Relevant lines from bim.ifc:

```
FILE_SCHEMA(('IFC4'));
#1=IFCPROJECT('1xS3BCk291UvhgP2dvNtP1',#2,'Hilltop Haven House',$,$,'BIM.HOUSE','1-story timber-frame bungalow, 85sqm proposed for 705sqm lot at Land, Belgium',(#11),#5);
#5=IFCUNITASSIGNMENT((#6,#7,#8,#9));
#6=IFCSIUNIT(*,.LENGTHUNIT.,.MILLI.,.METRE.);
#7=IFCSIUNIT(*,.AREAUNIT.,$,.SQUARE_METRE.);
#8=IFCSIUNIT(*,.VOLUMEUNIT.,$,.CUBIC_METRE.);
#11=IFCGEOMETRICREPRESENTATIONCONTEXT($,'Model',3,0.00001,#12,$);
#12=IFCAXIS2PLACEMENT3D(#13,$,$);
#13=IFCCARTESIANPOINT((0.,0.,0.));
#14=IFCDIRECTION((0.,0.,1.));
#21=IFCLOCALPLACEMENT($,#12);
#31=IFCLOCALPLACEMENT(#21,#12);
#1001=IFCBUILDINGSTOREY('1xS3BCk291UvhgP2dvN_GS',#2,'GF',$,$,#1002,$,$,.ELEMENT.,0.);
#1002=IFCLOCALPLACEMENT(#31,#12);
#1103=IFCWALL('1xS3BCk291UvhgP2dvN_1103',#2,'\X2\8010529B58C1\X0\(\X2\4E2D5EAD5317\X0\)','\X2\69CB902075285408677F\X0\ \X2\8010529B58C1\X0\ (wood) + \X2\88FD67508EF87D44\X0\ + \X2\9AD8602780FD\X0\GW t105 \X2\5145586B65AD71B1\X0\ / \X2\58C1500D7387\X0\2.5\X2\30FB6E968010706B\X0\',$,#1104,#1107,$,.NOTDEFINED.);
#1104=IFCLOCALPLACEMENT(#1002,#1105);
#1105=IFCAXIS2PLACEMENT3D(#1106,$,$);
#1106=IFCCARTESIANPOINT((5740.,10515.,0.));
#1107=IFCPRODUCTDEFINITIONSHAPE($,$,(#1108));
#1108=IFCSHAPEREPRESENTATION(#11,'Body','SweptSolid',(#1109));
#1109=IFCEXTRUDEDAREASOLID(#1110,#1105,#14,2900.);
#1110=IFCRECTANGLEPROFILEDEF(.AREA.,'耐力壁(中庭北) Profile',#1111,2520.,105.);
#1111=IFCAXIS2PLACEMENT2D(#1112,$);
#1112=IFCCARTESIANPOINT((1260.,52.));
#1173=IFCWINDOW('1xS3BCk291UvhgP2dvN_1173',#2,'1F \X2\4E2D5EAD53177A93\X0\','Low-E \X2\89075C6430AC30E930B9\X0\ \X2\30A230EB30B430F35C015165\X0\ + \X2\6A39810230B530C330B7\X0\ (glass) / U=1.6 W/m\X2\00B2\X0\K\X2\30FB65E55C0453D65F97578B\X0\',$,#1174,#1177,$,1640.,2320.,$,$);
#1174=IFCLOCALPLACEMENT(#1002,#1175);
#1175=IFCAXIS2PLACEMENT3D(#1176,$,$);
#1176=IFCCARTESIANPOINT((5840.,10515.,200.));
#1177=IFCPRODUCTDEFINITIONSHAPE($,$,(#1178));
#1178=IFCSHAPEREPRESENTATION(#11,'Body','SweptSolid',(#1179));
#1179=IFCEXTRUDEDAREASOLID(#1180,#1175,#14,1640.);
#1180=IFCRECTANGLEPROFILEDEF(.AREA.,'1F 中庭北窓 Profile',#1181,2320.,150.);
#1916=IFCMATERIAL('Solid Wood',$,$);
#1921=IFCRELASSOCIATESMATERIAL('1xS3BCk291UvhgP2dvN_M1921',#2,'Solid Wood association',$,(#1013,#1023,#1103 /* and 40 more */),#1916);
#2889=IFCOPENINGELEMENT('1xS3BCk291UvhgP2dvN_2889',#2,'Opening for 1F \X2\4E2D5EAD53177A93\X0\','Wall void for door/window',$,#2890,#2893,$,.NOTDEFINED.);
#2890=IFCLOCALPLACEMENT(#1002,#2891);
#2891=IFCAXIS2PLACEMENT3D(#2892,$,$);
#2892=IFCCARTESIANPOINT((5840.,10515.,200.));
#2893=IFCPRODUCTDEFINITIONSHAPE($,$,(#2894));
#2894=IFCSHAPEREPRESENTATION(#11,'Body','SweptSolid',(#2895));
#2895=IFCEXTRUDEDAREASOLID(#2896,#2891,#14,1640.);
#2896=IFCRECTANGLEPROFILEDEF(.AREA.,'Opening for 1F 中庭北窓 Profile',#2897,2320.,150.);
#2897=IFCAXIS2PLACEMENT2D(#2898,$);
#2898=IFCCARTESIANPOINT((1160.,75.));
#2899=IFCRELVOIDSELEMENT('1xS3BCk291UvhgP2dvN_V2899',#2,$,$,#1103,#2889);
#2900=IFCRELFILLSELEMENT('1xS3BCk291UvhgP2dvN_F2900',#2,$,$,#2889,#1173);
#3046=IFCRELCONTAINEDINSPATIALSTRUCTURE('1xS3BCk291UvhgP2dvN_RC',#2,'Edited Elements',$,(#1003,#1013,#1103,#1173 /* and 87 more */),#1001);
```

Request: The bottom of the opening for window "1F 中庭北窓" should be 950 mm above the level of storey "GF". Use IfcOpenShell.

```python
import numpy as np
import ifcopenshell
import ifcopenshell.api.geometry
import ifcopenshell.geom
import ifcopenshell.util.element
import ifcopenshell.util.placement
import ifcopenshell.util.shape
import ifcopenshell.util.unit

model = ifcopenshell.open("bim.ifc")
unit_scale = ifcopenshell.util.unit.calculate_unit_scale(model)

window = model.by_guid("1xS3BCk291UvhgP2dvN_1173")
opening = window.FillsVoids[0].RelatingOpeningElement
storey = ifcopenshell.util.element.get_container(window, ifc_class="IfcBuildingStorey")
level = ifcopenshell.util.placement.get_local_placement(storey.ObjectPlacement)[2, 3]

# The opening's origin need not be at the sill, so measure its lowest point.
shape = ifcopenshell.geom.create_shape(ifcopenshell.geom.settings(), opening)
bottom = ifcopenshell.util.shape.get_shape_bottom_elevation(shape, shape.geometry) / unit_scale
dz = level + 950.0 - bottom

shift = np.array([0.0, 0.0, dz])
# The window is not placed relative to its opening, so move both.
for product in (opening, window):
    matrix = ifcopenshell.util.placement.get_local_placement(product.ObjectPlacement)
    matrix[:3, 3] += shift
    ifcopenshell.api.geometry.edit_object_placement(model, product=product, matrix=matrix, is_si=False)

print(f"moved by {dz * unit_scale:+.3f} m")

model.write("bim_v2.ifc")
```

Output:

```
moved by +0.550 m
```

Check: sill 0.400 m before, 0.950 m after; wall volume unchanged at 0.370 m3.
